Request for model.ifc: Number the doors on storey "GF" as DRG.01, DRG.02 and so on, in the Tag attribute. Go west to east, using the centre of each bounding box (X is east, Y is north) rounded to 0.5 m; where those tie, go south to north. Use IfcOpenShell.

First a look at what the model holds.

```python
import ifcopenshell
import ifcopenshell.util.element
import ifcopenshell.util.placement

model = ifcopenshell.open("model.ifc")
print(model.schema)
storey = next(s for s in model.by_type("IfcBuildingStorey") if s.Name == "GF")
doors = [e for e in ifcopenshell.util.element.get_decomposition(storey) if e.is_a("IfcDoor")]
for e in sorted(doors, key=lambda e: e.id()):
    origin = ifcopenshell.util.placement.get_local_placement(e.ObjectPlacement)[:3, 3]
    print(e.id(), e.Tag, e.Name, origin.round(2) + 0.0, sep=" | ")
```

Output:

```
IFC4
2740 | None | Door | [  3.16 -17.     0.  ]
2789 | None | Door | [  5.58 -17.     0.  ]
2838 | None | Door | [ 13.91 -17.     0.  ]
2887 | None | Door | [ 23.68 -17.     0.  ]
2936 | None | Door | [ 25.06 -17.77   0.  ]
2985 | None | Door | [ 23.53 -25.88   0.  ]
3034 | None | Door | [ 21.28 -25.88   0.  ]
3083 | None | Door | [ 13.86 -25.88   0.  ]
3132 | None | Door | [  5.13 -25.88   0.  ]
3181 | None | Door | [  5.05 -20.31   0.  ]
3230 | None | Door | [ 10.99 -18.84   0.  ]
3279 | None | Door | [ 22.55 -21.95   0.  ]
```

```python
import ifcopenshell
import ifcopenshell.geom
import ifcopenshell.util.element
import ifcopenshell.util.shape

model = ifcopenshell.open("model.ifc")
settings = ifcopenshell.geom.settings()
settings.set("use-world-coords", True)


def centre(element):
    shape = ifcopenshell.geom.create_shape(settings, element)
    return ifcopenshell.util.shape.get_bbox_centroid(shape.geometry)


storey = next(s for s in model.by_type("IfcBuildingStorey") if s.Name == "GF")
doors = [e for e in ifcopenshell.util.element.get_decomposition(storey) if e.is_a("IfcDoor")]

# Insertion points can sit at a corner or the storey origin, so sort by the geometry (in metres).
centres = {e: centre(e) for e in doors}
doors.sort(key=lambda e: (round(centres[e][0] / 0.5), centres[e][1]))

for i, e in enumerate(doors, start=1):
    number = f"DRG.{i:02d}"
    e.Tag = number
    print(e.id(), number)

model.write("model_edited.ifc")
```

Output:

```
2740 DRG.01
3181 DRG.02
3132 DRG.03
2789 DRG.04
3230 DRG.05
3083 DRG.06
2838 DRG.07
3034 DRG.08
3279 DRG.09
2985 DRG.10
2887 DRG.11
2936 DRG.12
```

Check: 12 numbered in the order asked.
